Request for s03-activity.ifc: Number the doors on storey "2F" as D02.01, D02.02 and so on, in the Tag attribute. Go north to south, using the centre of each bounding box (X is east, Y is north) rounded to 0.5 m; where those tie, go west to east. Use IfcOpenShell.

First a look at what the model holds.

```python
import ifcopenshell
import ifcopenshell.util.element
import ifcopenshell.util.placement

model = ifcopenshell.open("s03-activity.ifc")
print(model.schema)
storey = next(s for s in model.by_type("IfcBuildingStorey") if s.Name == "2F")
doors = [e for e in ifcopenshell.util.element.get_decomposition(storey) if e.is_a("IfcDoor")]
for e in sorted(doors, key=lambda e: e.id()):
    origin = ifcopenshell.util.placement.get_local_placement(e.ObjectPlacement)[:3, 3]
    print(e.id(), e.Tag, e.Name, origin.round(2) + 0.0, sep=" | ")
```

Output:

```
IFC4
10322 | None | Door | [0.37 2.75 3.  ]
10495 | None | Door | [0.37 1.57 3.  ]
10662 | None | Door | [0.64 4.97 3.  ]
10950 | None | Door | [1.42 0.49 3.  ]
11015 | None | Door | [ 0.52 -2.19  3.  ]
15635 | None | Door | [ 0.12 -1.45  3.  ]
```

```python
import ifcopenshell
import ifcopenshell.geom
import ifcopenshell.util.element
import ifcopenshell.util.shape

model = ifcopenshell.open("s03-activity.ifc")
settings = ifcopenshell.geom.settings()
settings.set("use-world-coords", True)


def centre(element):
    shape = ifcopenshell.geom.create_shape(settings, element)
    return ifcopenshell.util.shape.get_bbox_centroid(shape.geometry)


storey = next(s for s in model.by_type("IfcBuildingStorey") if s.Name == "2F")
doors = [e for e in ifcopenshell.util.element.get_decomposition(storey) if e.is_a("IfcDoor")]

# Insertion points can sit at a corner or the storey origin, so sort by the geometry (in metres).
centres = {e: centre(e) for e in doors}
doors.sort(key=lambda e: (-round(centres[e][1] / 0.5), centres[e][0]))

for i, e in enumerate(doors, start=1):
    number = f"D02.{i:02d}"
    e.Tag = number
    print(e.id(), number)

model.write("s03-activity_edited.ifc")
```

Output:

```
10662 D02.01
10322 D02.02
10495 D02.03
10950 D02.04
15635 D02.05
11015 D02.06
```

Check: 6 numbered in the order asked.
